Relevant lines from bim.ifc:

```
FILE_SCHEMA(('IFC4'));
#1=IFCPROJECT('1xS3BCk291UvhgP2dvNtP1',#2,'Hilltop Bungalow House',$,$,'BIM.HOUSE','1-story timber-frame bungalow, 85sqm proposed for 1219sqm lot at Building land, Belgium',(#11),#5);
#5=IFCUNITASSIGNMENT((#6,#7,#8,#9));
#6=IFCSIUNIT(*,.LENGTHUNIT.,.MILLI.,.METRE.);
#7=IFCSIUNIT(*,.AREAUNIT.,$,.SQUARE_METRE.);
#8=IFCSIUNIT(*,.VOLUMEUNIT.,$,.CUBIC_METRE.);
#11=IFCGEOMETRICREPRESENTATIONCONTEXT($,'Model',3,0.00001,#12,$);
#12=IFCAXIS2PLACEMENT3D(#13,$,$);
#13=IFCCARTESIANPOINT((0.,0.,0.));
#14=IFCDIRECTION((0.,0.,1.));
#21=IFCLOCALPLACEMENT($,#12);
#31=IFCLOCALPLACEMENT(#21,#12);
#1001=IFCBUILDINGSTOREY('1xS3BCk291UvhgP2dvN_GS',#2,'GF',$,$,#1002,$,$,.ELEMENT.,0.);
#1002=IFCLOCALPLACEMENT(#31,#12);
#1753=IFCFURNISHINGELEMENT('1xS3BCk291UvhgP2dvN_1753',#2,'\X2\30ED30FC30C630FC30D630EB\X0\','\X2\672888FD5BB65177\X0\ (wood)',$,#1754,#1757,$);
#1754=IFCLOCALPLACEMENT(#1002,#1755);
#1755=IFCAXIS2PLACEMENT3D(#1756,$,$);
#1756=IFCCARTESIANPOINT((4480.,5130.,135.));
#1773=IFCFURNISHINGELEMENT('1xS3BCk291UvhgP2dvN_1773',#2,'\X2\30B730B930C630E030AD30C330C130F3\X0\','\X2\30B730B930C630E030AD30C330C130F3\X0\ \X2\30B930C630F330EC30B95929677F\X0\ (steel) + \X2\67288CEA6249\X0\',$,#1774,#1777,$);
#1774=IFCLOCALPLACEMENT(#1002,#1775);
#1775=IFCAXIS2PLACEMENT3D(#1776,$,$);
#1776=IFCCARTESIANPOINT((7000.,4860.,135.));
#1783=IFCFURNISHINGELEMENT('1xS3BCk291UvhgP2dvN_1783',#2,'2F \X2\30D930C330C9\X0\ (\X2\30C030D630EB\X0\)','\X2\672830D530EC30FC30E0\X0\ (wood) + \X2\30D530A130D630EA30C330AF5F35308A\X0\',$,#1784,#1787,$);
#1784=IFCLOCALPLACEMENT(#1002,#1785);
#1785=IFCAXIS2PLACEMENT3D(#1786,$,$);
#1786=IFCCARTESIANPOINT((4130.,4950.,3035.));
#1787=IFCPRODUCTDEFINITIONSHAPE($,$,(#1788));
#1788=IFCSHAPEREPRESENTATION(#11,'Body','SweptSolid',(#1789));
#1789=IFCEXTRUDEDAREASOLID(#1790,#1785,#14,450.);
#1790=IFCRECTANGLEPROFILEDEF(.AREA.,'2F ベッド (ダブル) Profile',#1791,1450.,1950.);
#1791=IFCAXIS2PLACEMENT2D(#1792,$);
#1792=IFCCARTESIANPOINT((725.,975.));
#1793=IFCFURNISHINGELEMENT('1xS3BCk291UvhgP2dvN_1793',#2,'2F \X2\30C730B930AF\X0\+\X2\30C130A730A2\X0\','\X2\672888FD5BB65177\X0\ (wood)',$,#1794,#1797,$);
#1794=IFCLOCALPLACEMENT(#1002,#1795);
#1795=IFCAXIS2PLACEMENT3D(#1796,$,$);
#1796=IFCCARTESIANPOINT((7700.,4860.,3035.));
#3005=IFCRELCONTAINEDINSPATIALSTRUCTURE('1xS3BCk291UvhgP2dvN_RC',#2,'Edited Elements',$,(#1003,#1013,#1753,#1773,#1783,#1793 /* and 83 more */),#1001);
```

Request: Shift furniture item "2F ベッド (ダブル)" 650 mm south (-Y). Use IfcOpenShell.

```python
import ifcopenshell
import ifcopenshell.api.geometry
import ifcopenshell.util.placement
import ifcopenshell.util.unit

model = ifcopenshell.open("bim.ifc")
unit_scale = ifcopenshell.util.unit.calculate_unit_scale(model)

item = model.by_id(1783)
matrix = ifcopenshell.util.placement.get_local_placement(item.ObjectPlacement)
matrix[1, 3] -= 0.65 / unit_scale
ifcopenshell.api.geometry.edit_object_placement(model, product=item, matrix=matrix, is_si=False)

print(ifcopenshell.util.placement.get_local_placement(item.ObjectPlacement).round(3) + 0.0)

model.write("bim_edited.ifc")
```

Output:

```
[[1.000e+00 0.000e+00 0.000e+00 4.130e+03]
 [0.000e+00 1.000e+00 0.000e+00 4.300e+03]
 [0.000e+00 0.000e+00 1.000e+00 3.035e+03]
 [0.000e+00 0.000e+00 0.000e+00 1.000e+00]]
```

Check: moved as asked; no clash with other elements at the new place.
